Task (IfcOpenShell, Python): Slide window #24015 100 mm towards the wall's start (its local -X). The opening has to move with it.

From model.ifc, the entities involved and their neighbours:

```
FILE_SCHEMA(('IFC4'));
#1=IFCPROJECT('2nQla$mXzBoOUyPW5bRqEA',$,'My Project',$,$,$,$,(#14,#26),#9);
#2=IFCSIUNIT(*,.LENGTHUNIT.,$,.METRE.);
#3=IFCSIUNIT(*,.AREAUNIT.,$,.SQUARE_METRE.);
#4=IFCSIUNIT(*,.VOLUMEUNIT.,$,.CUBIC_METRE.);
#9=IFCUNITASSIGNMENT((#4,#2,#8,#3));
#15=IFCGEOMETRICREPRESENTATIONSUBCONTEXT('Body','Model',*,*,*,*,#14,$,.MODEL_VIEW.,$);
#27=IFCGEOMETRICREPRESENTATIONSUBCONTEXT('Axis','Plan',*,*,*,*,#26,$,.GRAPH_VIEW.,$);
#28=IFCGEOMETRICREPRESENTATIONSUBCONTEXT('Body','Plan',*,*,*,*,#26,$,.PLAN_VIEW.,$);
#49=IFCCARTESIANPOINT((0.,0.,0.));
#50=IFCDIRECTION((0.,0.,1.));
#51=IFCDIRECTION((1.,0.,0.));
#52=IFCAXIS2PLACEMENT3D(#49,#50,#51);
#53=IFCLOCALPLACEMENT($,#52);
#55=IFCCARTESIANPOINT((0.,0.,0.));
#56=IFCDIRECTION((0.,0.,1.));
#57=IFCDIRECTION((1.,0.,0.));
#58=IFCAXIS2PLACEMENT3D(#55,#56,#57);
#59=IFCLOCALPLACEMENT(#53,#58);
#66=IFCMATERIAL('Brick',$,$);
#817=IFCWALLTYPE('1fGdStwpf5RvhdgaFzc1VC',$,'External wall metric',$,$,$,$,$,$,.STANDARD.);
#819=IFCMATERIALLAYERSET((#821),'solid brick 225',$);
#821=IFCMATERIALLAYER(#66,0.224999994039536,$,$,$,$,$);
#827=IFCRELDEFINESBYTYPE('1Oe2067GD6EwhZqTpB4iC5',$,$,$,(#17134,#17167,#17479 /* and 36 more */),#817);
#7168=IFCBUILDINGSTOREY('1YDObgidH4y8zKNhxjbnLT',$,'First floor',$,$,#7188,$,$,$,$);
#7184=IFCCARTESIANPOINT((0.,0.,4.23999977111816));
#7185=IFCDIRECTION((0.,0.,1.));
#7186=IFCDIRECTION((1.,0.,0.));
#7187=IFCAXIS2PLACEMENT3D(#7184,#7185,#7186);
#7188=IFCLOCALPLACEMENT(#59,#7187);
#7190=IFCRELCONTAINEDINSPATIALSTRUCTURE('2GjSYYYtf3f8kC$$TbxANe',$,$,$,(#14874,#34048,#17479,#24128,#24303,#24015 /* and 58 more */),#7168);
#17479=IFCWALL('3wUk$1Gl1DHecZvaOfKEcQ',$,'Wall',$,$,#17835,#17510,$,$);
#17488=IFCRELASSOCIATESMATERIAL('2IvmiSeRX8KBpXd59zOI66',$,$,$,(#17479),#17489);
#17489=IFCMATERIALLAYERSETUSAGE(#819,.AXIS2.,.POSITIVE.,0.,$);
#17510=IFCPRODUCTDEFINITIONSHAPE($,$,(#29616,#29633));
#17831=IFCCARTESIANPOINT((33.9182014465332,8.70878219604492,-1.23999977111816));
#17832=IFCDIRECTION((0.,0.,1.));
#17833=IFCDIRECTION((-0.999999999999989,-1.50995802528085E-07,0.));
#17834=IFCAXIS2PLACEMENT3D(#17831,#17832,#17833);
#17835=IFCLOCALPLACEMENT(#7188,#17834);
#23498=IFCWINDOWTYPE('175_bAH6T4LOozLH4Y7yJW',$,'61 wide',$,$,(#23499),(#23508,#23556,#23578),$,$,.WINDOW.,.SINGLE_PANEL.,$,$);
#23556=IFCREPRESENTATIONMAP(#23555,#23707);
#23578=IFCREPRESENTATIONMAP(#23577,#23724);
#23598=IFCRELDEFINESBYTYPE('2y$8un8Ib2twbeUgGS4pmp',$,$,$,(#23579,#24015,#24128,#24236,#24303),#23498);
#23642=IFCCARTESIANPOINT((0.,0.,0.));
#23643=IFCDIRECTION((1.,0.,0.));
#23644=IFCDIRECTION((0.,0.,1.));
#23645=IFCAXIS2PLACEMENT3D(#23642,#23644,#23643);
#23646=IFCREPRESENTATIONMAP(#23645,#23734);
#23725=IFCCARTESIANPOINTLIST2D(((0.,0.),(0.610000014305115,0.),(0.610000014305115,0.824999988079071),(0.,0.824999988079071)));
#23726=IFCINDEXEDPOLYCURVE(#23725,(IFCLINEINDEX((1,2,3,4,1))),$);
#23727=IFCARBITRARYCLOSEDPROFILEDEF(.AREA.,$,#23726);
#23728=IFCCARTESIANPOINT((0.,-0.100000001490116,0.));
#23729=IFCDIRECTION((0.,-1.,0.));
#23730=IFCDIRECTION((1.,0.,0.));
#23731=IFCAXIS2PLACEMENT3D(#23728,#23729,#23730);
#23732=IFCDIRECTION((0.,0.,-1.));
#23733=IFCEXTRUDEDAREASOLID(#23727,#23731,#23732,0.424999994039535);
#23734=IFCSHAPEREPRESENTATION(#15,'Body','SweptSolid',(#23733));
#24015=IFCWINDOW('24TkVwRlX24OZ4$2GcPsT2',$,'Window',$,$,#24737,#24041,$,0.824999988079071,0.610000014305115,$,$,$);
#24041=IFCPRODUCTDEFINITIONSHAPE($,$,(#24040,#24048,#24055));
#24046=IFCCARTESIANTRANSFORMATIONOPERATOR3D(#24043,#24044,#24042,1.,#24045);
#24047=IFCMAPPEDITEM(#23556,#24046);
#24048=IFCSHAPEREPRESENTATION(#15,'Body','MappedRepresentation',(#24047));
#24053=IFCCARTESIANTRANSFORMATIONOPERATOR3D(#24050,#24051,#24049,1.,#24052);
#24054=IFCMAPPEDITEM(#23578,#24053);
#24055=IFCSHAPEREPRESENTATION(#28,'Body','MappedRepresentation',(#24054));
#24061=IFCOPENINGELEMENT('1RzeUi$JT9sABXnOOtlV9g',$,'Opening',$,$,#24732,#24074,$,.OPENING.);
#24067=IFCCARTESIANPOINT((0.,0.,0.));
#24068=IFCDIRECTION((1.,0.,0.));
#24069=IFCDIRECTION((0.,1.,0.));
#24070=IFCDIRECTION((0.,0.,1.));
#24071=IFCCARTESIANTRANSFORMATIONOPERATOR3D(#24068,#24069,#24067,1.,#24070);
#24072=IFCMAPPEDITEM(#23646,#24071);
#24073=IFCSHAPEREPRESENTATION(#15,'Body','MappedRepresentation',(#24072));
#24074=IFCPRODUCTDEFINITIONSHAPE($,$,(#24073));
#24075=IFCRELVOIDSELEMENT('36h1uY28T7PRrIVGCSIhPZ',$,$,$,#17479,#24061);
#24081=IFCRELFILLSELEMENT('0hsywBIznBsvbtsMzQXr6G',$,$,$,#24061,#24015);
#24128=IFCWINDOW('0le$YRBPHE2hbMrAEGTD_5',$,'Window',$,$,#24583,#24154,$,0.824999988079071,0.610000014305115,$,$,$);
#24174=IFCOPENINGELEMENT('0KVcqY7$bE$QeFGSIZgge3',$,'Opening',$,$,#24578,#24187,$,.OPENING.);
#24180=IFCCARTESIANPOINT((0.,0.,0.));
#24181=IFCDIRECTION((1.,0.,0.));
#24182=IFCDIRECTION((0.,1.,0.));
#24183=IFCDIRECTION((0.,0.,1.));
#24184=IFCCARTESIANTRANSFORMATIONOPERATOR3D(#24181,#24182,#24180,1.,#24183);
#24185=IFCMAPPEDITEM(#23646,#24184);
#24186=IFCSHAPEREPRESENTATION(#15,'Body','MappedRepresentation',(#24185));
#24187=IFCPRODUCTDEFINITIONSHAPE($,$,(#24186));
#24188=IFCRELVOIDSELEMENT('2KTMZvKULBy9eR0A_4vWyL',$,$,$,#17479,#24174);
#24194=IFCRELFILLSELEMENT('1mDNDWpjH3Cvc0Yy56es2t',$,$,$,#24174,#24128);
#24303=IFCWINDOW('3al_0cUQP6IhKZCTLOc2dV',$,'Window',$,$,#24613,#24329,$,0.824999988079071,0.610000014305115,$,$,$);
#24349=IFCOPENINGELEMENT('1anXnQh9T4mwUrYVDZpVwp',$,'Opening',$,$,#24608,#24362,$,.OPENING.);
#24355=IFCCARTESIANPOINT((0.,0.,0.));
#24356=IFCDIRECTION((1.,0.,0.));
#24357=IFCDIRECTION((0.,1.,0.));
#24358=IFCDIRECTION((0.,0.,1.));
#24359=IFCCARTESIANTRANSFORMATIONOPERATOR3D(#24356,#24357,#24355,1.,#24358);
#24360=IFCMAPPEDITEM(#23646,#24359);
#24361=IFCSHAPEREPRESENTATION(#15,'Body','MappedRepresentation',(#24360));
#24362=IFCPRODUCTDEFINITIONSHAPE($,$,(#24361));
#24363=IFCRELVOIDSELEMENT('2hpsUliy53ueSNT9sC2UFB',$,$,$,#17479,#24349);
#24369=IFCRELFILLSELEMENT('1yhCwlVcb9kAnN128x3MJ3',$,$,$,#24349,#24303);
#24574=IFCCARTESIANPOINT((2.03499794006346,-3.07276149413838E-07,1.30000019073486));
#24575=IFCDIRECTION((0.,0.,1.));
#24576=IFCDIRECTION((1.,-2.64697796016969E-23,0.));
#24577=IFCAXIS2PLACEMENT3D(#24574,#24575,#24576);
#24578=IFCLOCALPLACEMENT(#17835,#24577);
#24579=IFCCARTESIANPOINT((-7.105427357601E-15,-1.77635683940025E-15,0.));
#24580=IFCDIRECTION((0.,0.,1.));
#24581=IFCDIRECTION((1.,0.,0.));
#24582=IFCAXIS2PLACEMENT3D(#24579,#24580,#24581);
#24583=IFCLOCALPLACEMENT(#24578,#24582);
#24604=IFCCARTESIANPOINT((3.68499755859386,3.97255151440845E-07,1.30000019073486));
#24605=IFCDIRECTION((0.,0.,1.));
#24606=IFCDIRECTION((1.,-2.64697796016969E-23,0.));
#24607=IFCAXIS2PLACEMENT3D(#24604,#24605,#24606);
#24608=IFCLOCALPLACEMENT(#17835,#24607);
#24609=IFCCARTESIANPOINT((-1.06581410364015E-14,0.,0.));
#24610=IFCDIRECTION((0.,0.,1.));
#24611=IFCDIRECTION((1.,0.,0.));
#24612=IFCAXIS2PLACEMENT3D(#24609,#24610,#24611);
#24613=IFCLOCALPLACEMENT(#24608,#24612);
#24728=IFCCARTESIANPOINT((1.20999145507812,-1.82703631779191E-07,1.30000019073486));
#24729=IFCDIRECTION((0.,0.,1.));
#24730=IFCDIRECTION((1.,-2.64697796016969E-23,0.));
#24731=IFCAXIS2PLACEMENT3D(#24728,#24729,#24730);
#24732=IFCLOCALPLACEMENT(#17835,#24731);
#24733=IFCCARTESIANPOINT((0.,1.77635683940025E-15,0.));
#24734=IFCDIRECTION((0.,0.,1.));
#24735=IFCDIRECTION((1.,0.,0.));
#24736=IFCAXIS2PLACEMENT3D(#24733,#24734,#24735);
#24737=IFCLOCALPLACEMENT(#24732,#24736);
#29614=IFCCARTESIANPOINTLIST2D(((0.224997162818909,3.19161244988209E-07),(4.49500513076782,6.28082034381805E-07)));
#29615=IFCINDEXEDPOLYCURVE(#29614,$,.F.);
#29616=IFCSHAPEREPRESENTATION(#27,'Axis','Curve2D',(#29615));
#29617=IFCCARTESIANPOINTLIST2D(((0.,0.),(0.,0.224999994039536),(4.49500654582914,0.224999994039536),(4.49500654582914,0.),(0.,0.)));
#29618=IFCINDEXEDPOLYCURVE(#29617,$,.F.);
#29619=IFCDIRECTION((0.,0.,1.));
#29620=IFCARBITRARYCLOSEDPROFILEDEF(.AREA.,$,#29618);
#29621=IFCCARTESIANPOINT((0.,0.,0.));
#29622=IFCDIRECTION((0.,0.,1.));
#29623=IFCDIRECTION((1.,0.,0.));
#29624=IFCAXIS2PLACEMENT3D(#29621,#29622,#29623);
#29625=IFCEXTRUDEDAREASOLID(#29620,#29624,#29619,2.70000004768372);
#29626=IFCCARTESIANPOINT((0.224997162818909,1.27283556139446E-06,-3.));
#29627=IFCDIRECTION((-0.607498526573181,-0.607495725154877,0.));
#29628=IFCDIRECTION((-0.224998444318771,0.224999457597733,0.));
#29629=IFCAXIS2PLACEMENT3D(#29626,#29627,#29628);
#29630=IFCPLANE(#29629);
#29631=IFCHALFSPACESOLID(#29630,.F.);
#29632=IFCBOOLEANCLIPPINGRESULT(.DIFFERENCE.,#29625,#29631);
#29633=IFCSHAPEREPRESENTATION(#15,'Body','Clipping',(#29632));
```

```python
import ifcopenshell
import ifcopenshell.api.geometry
import ifcopenshell.util.placement
import ifcopenshell.util.unit

model = ifcopenshell.open("model.ifc")
unit_scale = ifcopenshell.util.unit.calculate_unit_scale(model)

window = model.by_guid("24TkVwRlX24OZ4$2GcPsT2")
opening = window.FillsVoids[0].RelatingOpeningElement
wall = opening.VoidsElements[0].RelatingBuildingElement

wall_matrix = ifcopenshell.util.placement.get_local_placement(wall.ObjectPlacement)
shift = wall_matrix[:3, 0] * -0.1 / unit_scale
before = ifcopenshell.util.placement.get_local_placement(window.ObjectPlacement)[:3, 3].copy()

# The window is placed relative to its opening, so it follows when the opening moves.
matrix = ifcopenshell.util.placement.get_local_placement(opening.ObjectPlacement)
matrix[:3, 3] += shift
ifcopenshell.api.geometry.edit_object_placement(
    model, product=opening, matrix=matrix, is_si=False, should_transform_children=True
)

after = ifcopenshell.util.placement.get_local_placement(window.ObjectPlacement)[:3, 3]
print("window moved by", (after - before).round(3) + 0.0)

model.write("model_v2.ifc")
```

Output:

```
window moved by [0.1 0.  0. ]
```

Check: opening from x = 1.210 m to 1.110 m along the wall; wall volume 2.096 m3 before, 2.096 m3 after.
